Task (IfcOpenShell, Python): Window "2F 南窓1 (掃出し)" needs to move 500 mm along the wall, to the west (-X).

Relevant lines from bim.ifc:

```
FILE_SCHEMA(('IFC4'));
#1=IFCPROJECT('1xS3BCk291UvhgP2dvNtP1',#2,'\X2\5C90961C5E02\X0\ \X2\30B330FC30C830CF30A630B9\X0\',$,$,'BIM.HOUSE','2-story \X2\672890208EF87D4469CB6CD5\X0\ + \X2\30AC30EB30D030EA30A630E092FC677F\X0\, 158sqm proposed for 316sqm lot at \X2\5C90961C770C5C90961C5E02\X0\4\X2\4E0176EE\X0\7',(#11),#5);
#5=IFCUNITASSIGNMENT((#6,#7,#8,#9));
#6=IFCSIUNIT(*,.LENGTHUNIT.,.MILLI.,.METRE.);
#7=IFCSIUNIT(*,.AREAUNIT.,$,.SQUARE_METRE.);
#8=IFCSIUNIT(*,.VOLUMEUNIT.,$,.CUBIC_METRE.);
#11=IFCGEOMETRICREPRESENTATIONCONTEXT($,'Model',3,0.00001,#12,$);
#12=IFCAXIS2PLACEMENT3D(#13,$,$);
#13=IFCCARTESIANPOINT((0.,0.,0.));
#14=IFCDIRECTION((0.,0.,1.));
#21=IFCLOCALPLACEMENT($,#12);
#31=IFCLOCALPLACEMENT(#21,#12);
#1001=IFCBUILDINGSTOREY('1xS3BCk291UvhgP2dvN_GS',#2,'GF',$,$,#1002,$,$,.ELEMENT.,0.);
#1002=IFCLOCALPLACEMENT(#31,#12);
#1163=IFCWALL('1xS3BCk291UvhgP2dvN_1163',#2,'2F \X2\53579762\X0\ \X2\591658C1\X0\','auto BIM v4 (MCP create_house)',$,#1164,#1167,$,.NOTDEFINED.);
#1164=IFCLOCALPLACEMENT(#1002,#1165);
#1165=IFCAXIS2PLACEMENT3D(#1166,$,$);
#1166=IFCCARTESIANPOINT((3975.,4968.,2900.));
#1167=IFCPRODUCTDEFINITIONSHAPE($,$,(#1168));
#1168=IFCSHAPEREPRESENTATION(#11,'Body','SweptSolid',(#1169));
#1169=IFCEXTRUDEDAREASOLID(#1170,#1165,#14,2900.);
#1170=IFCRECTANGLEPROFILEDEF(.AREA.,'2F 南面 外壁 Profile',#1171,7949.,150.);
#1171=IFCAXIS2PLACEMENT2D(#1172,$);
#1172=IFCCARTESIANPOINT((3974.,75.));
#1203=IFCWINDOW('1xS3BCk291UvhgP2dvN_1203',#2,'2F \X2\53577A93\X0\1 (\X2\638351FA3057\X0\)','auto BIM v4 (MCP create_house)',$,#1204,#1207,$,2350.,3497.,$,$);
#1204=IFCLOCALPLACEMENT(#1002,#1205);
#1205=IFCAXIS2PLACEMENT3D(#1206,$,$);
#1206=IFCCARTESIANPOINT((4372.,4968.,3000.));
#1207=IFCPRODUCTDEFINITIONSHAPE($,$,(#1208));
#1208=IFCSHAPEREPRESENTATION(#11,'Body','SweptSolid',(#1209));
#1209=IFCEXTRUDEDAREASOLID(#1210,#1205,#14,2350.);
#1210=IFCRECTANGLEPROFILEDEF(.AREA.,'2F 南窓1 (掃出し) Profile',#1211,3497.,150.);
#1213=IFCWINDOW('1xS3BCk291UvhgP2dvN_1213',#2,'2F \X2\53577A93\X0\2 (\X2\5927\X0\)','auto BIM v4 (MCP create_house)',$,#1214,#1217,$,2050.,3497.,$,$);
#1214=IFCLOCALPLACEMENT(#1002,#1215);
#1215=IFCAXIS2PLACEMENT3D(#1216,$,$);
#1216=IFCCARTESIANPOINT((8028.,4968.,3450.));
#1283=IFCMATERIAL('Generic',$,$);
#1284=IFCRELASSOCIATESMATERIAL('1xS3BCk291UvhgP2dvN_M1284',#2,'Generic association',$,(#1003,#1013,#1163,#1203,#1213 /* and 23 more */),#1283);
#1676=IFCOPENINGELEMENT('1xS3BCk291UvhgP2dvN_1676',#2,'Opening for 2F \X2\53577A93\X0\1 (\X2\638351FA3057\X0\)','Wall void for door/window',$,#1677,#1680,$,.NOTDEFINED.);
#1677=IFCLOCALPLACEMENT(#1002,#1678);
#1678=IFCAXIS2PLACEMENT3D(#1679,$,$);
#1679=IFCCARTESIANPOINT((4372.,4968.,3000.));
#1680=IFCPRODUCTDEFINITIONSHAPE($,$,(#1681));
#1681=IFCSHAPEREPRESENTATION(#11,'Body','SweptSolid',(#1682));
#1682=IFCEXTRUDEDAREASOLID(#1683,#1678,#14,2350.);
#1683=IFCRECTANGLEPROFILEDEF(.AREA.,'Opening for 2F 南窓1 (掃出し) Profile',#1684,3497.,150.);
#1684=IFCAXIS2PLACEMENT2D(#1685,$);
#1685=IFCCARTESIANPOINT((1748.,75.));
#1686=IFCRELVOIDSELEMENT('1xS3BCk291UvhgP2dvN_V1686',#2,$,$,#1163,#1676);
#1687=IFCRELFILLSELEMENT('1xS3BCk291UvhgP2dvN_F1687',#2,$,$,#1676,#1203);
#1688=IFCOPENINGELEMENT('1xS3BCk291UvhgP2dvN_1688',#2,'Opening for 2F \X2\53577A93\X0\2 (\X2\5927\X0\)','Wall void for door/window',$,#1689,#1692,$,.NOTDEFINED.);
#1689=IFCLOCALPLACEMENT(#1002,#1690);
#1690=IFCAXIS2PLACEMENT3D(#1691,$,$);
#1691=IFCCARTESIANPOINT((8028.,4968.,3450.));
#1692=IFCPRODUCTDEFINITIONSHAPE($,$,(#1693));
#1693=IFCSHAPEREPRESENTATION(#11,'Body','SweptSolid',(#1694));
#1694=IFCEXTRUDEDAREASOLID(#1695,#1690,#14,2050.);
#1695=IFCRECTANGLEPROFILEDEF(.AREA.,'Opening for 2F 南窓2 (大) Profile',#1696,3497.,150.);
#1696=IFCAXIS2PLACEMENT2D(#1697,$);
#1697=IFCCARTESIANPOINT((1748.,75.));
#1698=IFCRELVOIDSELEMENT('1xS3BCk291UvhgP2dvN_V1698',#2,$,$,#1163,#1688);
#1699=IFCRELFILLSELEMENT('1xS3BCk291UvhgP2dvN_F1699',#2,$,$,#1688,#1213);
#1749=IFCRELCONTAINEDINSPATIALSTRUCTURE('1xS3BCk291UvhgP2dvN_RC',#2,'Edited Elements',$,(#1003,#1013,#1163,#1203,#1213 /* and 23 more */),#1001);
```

```python
import ifcopenshell
import ifcopenshell.api.geometry
import ifcopenshell.util.placement
import ifcopenshell.util.unit

model = ifcopenshell.open("bim.ifc")
unit_scale = ifcopenshell.util.unit.calculate_unit_scale(model)

window = model.by_id(1203)
opening = window.FillsVoids[0].RelatingOpeningElement
wall = opening.VoidsElements[0].RelatingBuildingElement

wall_matrix = ifcopenshell.util.placement.get_local_placement(wall.ObjectPlacement)
shift = wall_matrix[:3, 0] * -0.5 / unit_scale
before = ifcopenshell.util.placement.get_local_placement(window.ObjectPlacement)[:3, 3].copy()

# The window is not placed relative to its opening, so move both.
for product in (opening, window):
    matrix = ifcopenshell.util.placement.get_local_placement(product.ObjectPlacement)
    matrix[:3, 3] += shift
    ifcopenshell.api.geometry.edit_object_placement(model, product=product, matrix=matrix, is_si=False)

after = ifcopenshell.util.placement.get_local_placement(window.ObjectPlacement)[:3, 3]
print("window moved by", (after - before).round(3) + 0.0)

model.write("bim_updated.ifc")
```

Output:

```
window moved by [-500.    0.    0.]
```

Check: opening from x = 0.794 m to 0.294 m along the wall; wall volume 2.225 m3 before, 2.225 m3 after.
